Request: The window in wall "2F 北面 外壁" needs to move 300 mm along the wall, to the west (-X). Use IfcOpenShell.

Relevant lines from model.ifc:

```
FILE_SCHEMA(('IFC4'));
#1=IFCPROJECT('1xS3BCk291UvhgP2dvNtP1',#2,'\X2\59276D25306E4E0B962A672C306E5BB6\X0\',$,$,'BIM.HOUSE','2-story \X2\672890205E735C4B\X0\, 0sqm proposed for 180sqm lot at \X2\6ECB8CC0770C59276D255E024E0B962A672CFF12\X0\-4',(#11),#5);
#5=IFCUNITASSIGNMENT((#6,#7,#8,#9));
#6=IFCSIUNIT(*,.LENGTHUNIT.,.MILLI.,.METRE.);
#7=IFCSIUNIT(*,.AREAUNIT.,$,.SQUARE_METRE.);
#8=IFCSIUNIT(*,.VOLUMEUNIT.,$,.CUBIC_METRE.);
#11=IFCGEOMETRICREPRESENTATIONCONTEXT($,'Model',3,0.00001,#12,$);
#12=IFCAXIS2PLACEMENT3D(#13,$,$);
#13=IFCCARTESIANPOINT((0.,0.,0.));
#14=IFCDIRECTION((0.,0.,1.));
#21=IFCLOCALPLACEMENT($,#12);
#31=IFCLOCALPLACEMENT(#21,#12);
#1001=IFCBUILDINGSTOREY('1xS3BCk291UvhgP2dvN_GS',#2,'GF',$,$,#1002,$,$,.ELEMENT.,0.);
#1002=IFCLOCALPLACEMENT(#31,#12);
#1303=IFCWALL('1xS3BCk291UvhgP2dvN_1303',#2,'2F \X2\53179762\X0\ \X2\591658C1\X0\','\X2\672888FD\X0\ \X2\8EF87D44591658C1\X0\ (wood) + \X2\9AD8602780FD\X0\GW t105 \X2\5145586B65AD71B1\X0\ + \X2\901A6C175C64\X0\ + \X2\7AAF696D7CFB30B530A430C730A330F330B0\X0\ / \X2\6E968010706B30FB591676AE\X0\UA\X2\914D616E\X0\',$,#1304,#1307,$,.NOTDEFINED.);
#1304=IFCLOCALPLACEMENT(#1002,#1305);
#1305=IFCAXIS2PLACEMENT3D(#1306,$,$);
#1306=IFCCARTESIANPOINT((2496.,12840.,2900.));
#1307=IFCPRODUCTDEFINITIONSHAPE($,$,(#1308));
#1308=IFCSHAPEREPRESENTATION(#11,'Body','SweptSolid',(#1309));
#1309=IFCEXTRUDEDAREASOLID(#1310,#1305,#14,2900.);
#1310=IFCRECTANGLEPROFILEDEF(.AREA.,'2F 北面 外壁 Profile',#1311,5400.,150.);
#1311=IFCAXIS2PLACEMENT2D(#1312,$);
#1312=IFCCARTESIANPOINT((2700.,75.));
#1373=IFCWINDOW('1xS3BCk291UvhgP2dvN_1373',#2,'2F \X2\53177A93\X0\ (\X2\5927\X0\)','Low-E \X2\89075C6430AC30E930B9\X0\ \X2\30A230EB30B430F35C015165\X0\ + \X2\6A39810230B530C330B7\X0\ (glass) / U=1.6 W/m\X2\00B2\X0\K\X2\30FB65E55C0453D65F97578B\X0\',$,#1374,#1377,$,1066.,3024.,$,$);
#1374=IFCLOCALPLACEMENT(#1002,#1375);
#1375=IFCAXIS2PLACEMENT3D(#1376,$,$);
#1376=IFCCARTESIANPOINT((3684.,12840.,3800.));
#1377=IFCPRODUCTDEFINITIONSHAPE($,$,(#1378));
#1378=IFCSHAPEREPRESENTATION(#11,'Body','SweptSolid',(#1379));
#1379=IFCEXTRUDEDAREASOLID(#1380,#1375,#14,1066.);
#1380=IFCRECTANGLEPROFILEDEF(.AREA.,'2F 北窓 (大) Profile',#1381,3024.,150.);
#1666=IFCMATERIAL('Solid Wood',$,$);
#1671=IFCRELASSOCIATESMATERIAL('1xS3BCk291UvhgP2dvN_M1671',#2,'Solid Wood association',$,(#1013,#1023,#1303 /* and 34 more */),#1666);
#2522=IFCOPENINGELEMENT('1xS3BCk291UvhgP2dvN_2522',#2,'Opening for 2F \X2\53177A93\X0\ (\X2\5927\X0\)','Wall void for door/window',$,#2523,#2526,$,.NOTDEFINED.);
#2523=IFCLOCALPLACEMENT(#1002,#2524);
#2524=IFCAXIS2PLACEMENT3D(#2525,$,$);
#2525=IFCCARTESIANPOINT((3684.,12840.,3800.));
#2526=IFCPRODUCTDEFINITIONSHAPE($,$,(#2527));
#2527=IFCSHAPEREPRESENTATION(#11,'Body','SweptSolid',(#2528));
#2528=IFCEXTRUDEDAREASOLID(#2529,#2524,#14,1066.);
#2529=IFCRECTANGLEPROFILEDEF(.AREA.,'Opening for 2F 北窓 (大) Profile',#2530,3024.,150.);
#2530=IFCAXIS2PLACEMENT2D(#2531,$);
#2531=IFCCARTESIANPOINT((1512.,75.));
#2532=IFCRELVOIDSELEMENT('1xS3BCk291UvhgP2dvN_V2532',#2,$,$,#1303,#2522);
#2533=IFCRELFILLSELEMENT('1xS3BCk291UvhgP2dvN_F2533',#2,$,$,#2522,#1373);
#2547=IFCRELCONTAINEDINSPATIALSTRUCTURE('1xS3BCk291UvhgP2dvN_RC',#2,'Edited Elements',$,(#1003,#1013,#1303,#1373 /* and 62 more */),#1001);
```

```python
import ifcopenshell
import ifcopenshell.api.geometry
import ifcopenshell.util.placement

model = ifcopenshell.open("model.ifc")

window = model.by_guid("1xS3BCk291UvhgP2dvN_1373")
opening = window.FillsVoids[0].RelatingOpeningElement
wall = opening.VoidsElements[0].RelatingBuildingElement

wall_matrix = ifcopenshell.util.placement.get_local_placement(wall.ObjectPlacement)
shift = wall_matrix[:3, 0] * -300.0
before = ifcopenshell.util.placement.get_local_placement(window.ObjectPlacement)[:3, 3].copy()

# The window is not placed relative to its opening, so move both.
for product in (opening, window):
    matrix = ifcopenshell.util.placement.get_local_placement(product.ObjectPlacement)
    matrix[:3, 3] += shift
    ifcopenshell.api.geometry.edit_object_placement(model, product=product, matrix=matrix, is_si=False)

after = ifcopenshell.util.placement.get_local_placement(window.ObjectPlacement)[:3, 3]
print("window moved by", (after - before).round(3) + 0.0)

model.write("model_updated.ifc")
```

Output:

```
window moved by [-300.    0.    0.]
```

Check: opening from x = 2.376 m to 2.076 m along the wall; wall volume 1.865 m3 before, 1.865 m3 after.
